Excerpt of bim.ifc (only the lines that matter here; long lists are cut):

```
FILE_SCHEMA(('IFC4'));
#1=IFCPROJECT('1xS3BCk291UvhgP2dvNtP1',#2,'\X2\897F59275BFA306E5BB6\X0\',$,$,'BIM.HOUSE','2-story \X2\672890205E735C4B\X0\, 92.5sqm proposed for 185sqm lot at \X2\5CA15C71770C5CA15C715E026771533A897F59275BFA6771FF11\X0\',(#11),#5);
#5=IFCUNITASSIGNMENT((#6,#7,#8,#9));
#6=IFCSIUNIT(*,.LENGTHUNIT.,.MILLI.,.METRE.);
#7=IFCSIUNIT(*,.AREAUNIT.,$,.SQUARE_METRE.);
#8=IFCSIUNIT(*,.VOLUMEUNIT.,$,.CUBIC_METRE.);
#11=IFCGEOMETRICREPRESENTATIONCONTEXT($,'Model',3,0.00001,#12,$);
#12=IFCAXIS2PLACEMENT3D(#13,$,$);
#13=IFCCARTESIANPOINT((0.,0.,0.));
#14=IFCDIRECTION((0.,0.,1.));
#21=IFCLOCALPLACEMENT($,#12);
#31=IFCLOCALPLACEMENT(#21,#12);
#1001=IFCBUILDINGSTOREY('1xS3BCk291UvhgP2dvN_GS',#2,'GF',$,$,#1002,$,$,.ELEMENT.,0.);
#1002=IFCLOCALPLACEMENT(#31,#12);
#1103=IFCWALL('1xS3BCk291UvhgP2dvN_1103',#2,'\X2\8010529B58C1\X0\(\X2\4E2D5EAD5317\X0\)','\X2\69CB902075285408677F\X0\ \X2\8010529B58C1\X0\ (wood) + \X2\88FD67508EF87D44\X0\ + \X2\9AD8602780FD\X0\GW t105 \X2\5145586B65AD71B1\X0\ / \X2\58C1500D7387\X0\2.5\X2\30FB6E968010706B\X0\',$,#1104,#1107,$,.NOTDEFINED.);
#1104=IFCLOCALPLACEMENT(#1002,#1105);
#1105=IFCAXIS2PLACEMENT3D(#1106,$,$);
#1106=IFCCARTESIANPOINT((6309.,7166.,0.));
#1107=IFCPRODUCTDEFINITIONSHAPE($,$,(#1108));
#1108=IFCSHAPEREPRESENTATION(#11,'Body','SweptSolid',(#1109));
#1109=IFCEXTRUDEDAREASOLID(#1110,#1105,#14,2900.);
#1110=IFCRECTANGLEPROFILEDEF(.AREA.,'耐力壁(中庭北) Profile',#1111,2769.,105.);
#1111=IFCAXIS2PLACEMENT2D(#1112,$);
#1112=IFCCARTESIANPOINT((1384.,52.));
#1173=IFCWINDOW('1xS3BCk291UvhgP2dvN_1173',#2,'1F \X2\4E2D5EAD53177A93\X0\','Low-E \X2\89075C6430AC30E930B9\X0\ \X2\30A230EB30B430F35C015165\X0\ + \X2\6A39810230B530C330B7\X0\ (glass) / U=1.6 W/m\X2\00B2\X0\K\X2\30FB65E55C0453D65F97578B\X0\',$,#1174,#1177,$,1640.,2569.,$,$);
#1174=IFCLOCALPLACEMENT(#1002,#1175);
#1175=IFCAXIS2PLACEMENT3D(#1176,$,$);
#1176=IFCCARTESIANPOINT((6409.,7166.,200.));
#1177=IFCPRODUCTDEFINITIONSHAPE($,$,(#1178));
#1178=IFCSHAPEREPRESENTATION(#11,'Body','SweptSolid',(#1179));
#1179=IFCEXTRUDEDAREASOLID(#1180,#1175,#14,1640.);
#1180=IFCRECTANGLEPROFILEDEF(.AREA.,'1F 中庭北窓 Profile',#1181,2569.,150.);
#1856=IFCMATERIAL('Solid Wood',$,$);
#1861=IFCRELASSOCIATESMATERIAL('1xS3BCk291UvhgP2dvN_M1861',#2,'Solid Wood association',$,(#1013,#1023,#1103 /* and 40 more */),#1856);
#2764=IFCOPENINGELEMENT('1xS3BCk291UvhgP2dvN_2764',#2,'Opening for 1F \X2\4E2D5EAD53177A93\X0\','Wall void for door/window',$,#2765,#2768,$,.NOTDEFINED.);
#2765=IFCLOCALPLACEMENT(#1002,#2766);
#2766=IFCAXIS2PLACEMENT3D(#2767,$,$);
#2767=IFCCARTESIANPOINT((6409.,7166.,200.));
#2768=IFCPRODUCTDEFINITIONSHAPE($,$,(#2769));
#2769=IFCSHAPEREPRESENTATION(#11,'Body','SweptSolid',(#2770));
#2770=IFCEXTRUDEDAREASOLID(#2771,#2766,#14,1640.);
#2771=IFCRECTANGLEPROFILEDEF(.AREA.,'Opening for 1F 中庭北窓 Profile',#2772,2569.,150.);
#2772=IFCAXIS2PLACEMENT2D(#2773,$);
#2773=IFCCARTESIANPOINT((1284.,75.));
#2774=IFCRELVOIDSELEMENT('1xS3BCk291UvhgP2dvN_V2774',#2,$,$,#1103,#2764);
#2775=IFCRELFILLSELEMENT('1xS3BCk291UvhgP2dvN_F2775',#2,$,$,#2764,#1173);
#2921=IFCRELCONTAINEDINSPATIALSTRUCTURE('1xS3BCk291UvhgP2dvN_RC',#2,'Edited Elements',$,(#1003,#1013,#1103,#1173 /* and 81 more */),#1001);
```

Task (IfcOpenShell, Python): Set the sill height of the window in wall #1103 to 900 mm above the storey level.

```python
import numpy as np
import ifcopenshell
import ifcopenshell.api.geometry
import ifcopenshell.geom
import ifcopenshell.util.element
import ifcopenshell.util.placement
import ifcopenshell.util.shape
import ifcopenshell.util.unit

model = ifcopenshell.open("bim.ifc")
unit_scale = ifcopenshell.util.unit.calculate_unit_scale(model)

window = model.by_guid("1xS3BCk291UvhgP2dvN_1173")
opening = window.FillsVoids[0].RelatingOpeningElement
storey = ifcopenshell.util.element.get_container(window, ifc_class="IfcBuildingStorey")
level = ifcopenshell.util.placement.get_local_placement(storey.ObjectPlacement)[2, 3]

# The opening's origin need not be at the sill, so measure its lowest point.
shape = ifcopenshell.geom.create_shape(ifcopenshell.geom.settings(), opening)
bottom = ifcopenshell.util.shape.get_shape_bottom_elevation(shape, shape.geometry) / unit_scale
dz = level + 900.0 - bottom

shift = np.array([0.0, 0.0, dz])
# The window is not placed relative to its opening, so move both.
for product in (opening, window):
    matrix = ifcopenshell.util.placement.get_local_placement(product.ObjectPlacement)
    matrix[:3, 3] += shift
    ifcopenshell.api.geometry.edit_object_placement(model, product=product, matrix=matrix, is_si=False)

print(f"moved by {dz * unit_scale:+.3f} m")

model.write("bim_v2.ifc")
```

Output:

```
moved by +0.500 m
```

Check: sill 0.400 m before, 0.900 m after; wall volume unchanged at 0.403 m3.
